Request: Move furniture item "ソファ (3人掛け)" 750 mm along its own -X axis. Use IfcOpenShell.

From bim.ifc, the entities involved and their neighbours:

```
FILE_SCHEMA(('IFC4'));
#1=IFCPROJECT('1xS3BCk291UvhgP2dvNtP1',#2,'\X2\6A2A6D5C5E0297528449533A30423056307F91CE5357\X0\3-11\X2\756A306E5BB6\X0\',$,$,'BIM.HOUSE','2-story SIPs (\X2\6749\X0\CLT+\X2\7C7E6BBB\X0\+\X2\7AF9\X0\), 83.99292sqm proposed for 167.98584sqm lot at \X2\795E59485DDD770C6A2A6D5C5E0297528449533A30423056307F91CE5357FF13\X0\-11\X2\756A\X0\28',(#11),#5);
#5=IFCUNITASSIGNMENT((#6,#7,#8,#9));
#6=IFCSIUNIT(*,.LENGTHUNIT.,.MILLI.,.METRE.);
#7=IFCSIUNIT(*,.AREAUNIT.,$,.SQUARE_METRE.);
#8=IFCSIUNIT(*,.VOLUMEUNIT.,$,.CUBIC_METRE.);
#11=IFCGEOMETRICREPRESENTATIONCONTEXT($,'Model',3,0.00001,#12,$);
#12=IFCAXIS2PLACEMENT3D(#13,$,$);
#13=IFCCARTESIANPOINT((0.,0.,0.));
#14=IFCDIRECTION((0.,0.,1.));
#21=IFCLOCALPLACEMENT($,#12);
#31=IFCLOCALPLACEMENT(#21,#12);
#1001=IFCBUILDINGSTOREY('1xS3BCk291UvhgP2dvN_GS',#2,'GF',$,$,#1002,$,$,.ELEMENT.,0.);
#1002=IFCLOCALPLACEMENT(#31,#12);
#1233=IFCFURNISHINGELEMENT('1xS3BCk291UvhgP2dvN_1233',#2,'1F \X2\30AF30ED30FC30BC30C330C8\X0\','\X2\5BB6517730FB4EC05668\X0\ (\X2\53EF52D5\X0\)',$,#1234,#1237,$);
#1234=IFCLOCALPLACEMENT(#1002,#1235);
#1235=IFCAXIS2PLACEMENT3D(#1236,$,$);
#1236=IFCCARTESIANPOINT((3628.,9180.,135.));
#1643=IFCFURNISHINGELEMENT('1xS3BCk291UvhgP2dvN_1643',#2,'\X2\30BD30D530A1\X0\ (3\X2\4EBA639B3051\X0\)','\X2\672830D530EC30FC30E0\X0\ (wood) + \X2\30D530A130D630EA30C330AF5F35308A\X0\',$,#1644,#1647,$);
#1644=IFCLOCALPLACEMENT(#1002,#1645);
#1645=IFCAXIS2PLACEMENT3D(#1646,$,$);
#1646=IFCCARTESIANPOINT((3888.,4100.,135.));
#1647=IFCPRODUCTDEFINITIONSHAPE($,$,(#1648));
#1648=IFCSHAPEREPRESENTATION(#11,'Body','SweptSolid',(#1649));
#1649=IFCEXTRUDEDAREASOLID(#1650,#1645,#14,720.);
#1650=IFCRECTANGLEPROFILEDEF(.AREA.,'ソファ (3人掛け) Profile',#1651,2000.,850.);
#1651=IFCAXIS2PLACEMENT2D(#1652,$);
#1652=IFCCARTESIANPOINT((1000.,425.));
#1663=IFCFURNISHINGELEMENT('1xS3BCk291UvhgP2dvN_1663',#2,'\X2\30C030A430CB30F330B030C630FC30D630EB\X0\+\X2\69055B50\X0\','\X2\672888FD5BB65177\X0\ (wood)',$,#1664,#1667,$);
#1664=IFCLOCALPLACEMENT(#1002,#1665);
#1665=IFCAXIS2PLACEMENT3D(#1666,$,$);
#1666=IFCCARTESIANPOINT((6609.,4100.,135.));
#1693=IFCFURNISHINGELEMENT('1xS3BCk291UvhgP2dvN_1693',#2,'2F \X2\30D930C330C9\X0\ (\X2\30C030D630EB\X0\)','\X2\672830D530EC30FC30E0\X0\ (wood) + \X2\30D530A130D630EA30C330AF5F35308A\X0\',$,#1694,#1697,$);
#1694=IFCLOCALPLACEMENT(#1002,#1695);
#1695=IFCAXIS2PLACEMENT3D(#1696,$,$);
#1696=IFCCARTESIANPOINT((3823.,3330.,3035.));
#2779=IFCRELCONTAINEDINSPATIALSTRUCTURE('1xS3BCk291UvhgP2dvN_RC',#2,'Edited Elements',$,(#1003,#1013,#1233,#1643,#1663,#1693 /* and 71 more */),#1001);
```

```python
import ifcopenshell
import ifcopenshell.api.geometry
import ifcopenshell.util.placement
import ifcopenshell.util.unit

model = ifcopenshell.open("bim.ifc")
unit_scale = ifcopenshell.util.unit.calculate_unit_scale(model)

item = model.by_id(1643)
matrix = ifcopenshell.util.placement.get_local_placement(item.ObjectPlacement)
matrix[:3, 3] -= matrix[:3, 0] * 0.75 / unit_scale
ifcopenshell.api.geometry.edit_object_placement(model, product=item, matrix=matrix, is_si=False)

print(ifcopenshell.util.placement.get_local_placement(item.ObjectPlacement).round(3) + 0.0)

model.write("bim-out.ifc")
```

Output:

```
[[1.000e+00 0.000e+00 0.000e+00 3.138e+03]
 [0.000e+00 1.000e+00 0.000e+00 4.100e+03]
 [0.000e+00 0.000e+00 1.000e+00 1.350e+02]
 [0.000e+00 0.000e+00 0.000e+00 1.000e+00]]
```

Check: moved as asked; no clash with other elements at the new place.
